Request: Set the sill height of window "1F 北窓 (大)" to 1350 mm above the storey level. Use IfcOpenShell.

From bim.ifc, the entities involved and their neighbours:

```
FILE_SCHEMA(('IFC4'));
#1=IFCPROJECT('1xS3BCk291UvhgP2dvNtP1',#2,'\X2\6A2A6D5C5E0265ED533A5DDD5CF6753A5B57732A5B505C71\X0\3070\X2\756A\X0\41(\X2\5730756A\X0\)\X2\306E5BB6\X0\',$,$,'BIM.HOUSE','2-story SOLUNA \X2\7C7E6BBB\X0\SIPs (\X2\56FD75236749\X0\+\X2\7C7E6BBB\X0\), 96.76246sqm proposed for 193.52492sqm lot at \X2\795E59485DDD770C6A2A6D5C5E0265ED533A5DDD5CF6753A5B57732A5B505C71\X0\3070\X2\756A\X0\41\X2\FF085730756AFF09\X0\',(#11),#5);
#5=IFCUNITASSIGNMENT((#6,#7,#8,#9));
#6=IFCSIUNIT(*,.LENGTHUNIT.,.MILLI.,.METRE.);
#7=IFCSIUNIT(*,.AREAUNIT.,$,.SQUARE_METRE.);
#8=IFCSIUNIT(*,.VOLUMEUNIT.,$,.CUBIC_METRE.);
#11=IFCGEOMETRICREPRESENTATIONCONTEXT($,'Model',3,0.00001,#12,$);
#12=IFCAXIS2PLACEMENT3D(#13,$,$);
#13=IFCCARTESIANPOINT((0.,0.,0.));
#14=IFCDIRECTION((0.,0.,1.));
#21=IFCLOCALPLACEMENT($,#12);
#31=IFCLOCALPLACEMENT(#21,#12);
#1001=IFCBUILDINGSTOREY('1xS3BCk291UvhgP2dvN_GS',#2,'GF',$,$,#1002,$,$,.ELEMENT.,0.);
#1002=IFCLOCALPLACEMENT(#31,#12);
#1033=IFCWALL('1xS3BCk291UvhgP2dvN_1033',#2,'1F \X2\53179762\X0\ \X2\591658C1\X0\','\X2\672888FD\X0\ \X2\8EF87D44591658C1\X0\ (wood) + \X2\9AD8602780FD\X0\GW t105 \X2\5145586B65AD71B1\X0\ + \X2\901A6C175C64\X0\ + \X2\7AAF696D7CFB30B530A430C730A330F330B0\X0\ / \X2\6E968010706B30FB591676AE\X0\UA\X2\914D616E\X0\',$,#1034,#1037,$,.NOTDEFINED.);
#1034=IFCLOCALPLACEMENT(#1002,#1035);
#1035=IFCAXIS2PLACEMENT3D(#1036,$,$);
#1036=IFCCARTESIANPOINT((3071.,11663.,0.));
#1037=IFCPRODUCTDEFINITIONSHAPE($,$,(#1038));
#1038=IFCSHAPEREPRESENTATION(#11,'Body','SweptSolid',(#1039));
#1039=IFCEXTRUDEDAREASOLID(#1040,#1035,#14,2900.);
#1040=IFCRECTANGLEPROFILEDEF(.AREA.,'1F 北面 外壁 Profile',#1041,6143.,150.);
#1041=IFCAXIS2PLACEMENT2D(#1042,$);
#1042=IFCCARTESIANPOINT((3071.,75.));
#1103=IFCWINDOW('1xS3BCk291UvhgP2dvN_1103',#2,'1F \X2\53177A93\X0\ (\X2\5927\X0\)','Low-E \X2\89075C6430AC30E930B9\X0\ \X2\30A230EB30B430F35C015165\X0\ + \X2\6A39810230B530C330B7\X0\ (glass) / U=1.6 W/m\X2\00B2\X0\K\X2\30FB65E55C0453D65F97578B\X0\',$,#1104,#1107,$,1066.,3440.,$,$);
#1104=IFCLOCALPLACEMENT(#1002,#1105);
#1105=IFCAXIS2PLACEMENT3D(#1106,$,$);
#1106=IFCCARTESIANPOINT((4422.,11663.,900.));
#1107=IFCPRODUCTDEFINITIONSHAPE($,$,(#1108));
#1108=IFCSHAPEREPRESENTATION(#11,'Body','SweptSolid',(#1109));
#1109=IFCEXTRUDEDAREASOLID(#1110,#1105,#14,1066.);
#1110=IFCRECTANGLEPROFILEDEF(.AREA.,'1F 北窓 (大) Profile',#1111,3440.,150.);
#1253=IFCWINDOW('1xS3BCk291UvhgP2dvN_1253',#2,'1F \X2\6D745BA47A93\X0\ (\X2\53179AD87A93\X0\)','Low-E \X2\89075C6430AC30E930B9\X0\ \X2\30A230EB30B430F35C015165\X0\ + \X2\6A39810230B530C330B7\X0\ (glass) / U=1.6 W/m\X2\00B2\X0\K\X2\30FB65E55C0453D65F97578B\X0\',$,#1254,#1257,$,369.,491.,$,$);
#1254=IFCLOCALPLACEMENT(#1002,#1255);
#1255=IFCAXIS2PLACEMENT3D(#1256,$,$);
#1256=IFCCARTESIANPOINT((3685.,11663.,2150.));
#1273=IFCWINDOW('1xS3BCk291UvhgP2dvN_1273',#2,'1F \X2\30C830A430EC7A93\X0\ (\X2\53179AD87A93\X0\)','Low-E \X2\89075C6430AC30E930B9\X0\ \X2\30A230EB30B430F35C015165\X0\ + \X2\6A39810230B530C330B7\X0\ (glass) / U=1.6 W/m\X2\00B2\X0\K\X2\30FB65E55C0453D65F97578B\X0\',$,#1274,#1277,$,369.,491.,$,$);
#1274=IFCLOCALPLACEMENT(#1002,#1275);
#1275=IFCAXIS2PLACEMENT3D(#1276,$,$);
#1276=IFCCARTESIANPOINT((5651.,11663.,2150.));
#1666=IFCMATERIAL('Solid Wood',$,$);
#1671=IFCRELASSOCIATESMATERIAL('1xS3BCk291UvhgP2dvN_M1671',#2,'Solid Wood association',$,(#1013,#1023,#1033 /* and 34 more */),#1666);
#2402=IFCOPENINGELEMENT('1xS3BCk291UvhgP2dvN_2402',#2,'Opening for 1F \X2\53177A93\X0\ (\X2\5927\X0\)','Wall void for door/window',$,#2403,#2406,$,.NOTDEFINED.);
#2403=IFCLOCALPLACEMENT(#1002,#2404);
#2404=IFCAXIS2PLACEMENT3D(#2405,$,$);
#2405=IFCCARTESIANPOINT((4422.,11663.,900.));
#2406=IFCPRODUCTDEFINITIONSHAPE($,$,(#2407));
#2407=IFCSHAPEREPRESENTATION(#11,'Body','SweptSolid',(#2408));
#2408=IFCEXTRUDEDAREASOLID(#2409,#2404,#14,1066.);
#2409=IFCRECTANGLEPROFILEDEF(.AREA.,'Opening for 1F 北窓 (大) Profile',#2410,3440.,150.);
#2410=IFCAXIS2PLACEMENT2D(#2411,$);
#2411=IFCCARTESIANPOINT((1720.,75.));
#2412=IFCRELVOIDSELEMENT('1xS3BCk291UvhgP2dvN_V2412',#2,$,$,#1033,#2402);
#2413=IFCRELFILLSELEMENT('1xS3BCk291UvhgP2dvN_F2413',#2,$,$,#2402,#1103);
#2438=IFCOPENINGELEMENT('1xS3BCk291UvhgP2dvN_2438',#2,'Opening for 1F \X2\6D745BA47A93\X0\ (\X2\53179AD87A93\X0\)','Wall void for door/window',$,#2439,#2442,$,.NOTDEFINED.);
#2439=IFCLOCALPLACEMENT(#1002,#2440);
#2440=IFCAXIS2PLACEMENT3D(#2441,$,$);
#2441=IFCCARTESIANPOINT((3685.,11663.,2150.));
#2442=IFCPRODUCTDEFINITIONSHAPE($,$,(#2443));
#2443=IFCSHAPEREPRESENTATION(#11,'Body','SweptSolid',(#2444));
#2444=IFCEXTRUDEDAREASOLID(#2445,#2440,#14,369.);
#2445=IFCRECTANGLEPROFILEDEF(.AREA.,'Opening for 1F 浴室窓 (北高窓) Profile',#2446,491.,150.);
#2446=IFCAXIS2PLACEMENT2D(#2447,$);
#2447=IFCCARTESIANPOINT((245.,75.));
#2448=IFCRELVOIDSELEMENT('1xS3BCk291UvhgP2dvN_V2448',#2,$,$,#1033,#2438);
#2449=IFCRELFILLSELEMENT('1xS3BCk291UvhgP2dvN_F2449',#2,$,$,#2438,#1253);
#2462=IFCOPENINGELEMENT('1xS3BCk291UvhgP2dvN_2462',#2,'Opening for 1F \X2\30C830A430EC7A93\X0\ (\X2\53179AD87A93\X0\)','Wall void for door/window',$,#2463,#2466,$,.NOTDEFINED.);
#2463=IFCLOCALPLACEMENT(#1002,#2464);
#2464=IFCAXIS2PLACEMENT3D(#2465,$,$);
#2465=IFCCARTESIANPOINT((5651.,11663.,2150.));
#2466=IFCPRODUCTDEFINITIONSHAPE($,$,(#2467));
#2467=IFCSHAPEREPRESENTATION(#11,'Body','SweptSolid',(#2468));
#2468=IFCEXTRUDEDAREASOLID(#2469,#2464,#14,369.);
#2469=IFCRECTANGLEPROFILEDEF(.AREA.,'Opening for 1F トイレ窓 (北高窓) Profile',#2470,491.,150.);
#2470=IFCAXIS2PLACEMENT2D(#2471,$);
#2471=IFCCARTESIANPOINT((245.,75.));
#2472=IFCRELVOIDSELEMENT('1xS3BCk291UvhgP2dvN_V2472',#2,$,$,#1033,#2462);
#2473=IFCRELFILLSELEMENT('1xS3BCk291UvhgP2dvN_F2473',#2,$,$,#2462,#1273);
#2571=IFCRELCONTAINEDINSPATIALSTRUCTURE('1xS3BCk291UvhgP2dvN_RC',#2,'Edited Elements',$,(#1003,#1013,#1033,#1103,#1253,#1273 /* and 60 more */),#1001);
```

```python
import numpy as np
import ifcopenshell
import ifcopenshell.api.geometry
import ifcopenshell.geom
import ifcopenshell.util.element
import ifcopenshell.util.placement
import ifcopenshell.util.shape
import ifcopenshell.util.unit

model = ifcopenshell.open("bim.ifc")
unit_scale = ifcopenshell.util.unit.calculate_unit_scale(model)

window = model.by_id(1103)
opening = window.FillsVoids[0].RelatingOpeningElement
storey = ifcopenshell.util.element.get_container(window, ifc_class="IfcBuildingStorey")
level = ifcopenshell.util.placement.get_local_placement(storey.ObjectPlacement)[2, 3]

# The opening's origin need not be at the sill, so measure its lowest point.
shape = ifcopenshell.geom.create_shape(ifcopenshell.geom.settings(), opening)
bottom = ifcopenshell.util.shape.get_shape_bottom_elevation(shape, shape.geometry) / unit_scale
dz = level + 1350.0 - bottom

shift = np.array([0.0, 0.0, dz])
# The window is not placed relative to its opening, so move both.
for product in (opening, window):
    matrix = ifcopenshell.util.placement.get_local_placement(product.ObjectPlacement)
    matrix[:3, 3] += shift
    ifcopenshell.api.geometry.edit_object_placement(model, product=product, matrix=matrix, is_si=False)

print(f"moved by {dz * unit_scale:+.3f} m")

model.write("bim_edited.ifc")
```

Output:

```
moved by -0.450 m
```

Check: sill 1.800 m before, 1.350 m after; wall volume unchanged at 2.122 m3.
